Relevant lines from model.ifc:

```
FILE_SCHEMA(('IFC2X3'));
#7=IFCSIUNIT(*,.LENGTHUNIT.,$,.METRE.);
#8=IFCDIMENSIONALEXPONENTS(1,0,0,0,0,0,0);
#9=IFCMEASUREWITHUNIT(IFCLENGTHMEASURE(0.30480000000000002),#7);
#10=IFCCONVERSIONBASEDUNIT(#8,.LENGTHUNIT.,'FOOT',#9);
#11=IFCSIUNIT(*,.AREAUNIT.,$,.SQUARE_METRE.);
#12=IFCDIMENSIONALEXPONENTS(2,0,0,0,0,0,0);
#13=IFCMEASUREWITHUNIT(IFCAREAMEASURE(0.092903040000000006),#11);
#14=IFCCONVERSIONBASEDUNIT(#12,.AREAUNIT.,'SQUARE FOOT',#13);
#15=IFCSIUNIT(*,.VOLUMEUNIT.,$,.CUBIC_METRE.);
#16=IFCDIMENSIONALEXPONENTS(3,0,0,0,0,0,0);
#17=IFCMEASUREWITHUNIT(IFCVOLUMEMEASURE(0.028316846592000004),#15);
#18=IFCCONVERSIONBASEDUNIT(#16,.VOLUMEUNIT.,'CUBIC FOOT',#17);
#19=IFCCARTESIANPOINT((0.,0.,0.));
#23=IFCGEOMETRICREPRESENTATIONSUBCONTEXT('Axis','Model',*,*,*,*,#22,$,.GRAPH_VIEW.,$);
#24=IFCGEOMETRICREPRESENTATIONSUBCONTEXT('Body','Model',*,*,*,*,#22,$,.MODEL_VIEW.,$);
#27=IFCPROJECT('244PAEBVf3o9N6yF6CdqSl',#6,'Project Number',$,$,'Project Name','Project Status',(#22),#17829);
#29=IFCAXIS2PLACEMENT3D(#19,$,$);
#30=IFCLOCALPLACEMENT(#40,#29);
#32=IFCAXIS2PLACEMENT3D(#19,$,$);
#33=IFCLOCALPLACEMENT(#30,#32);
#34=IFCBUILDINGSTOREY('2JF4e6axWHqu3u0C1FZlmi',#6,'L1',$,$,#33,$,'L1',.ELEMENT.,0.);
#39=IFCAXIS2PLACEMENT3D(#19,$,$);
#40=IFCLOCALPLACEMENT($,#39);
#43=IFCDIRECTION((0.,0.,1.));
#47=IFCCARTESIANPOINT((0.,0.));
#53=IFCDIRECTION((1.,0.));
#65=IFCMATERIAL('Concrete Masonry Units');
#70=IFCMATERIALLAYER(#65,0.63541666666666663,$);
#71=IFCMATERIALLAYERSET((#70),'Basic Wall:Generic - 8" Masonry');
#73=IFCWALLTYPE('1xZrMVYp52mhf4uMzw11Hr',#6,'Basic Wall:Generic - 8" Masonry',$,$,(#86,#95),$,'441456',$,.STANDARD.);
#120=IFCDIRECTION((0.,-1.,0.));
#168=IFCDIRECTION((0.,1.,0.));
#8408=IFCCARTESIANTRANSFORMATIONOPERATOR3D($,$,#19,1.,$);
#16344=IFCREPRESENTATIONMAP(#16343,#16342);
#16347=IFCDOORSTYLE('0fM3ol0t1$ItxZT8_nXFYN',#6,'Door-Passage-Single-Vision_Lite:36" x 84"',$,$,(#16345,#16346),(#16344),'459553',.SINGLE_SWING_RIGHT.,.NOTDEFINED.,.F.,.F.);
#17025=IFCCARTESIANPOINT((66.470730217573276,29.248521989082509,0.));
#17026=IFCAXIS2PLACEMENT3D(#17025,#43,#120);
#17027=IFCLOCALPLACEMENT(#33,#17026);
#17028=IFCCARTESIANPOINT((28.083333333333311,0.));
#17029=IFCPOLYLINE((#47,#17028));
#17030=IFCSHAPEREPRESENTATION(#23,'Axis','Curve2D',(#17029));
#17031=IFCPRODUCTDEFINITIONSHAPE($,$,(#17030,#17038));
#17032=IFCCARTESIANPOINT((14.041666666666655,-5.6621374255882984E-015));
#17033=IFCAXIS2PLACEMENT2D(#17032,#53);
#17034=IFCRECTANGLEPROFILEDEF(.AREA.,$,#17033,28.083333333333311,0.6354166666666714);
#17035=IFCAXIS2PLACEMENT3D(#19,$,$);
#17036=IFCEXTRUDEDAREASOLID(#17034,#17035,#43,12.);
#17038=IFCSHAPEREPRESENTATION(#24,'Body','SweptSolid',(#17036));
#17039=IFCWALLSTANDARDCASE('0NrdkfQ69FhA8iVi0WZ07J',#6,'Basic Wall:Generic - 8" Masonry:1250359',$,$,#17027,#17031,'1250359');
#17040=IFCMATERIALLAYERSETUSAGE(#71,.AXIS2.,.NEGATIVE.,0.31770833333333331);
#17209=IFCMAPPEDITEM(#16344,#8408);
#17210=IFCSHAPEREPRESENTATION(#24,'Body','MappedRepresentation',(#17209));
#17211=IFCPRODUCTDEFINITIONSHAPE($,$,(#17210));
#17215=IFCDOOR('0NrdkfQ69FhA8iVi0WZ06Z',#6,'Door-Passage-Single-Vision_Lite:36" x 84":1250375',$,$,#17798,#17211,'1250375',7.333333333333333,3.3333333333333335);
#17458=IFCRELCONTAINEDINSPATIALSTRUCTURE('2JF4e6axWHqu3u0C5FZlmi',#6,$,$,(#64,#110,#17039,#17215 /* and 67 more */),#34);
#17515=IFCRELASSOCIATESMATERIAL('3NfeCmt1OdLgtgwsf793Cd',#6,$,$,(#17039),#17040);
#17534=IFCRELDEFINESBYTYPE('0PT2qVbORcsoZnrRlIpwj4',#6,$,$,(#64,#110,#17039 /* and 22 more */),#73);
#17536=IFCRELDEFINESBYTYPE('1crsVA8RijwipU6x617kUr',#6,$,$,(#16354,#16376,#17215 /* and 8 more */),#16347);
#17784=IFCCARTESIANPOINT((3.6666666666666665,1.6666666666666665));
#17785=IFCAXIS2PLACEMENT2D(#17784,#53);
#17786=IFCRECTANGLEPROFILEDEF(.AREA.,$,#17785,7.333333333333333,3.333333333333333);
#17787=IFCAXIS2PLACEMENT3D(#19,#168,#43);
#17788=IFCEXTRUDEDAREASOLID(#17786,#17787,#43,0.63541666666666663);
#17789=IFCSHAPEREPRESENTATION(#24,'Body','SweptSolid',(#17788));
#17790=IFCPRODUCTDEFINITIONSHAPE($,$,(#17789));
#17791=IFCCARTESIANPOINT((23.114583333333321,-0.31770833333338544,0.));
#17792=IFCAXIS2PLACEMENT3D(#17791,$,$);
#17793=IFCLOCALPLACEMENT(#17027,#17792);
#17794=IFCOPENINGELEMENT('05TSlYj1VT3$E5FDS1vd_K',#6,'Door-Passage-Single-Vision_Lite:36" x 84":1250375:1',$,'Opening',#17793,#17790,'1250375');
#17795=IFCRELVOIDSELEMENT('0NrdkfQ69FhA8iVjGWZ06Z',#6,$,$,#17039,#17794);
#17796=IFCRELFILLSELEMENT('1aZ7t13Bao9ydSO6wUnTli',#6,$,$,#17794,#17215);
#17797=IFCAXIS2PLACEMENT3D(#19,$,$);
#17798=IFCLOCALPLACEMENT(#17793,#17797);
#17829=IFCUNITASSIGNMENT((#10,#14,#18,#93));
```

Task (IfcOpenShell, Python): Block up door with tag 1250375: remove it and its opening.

```python
import ifcopenshell
import ifcopenshell.api.feature
import ifcopenshell.api.root
import ifcopenshell.geom
import ifcopenshell.util.shape

model = ifcopenshell.open("model.ifc")
settings = ifcopenshell.geom.settings()


def volume(element):
    """Net volume in cubic metres, openings subtracted."""
    shape = ifcopenshell.geom.create_shape(settings, element)
    return ifcopenshell.util.shape.get_volume(shape.geometry)


door = model.by_guid("0NrdkfQ69FhA8iVi0WZ06Z")
opening = door.FillsVoids[0].RelatingOpeningElement
wall = opening.VoidsElements[0].RelatingBuildingElement
before = volume(wall)

ifcopenshell.api.root.remove_product(model, product=door)
ifcopenshell.api.feature.remove_feature(model, feature=opening)

after = volume(wall)

print(f"wall volume {before:.3f} -> {after:.3f} m3")

model.write("model_rev.ifc")
```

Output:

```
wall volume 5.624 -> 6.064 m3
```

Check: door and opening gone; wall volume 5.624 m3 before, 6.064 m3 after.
